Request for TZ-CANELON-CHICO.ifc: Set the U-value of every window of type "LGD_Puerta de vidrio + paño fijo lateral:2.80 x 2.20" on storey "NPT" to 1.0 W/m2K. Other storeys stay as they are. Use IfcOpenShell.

First a look at what the model holds.

```python
import ifcopenshell
import ifcopenshell.util.element

model = ifcopenshell.open("TZ-CANELON-CHICO.ifc")
print(model.schema)
storey = next(s for s in model.by_type("IfcBuildingStorey") if s.Name == "NPT")
windows = [e for e in ifcopenshell.util.element.get_decomposition(storey) if e.is_a("IfcWindow")]
seen = {}
for e in windows:
    element_type = ifcopenshell.util.element.get_type(e)
    key = (element_type.Name if element_type != e and element_type else None, ifcopenshell.util.element.get_pset(e, "Pset_WindowCommon", "ThermalTransmittance"))
    seen[key] = seen.get(key, 0) + 1
for (name, value), count in sorted(seen.items(), key=str):
    print(count, "x", name, "|", value)
```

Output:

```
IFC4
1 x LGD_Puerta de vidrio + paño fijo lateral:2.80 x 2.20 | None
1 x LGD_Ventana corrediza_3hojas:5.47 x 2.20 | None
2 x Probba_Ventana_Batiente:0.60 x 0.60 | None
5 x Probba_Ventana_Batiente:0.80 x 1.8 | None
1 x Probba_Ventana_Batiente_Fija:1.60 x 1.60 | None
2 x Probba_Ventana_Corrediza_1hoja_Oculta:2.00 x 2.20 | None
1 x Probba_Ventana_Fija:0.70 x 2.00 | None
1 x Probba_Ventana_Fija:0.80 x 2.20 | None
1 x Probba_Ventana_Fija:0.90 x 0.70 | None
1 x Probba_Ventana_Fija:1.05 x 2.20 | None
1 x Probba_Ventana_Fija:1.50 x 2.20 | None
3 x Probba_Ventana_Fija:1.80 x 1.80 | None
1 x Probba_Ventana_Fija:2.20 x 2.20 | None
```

```python
import ifcopenshell
import ifcopenshell.api.pset
import ifcopenshell.util.element

model = ifcopenshell.open("TZ-CANELON-CHICO.ifc")

storey = next(s for s in model.by_type("IfcBuildingStorey") if s.Name == "NPT")
windows = [e for e in ifcopenshell.util.element.get_decomposition(storey) if e.is_a("IfcWindow")]

count = 0
for e in windows:
    element_type = ifcopenshell.util.element.get_type(e)
    if element_type in (None, e) or element_type.Name != "LGD_Puerta de vidrio + paño fijo lateral:2.80 x 2.20":
        continue
    # add_pset returns the element's existing set when there is one.
    pset = ifcopenshell.api.pset.add_pset(model, product=e, name="Pset_WindowCommon")
    ifcopenshell.api.pset.edit_pset(model, pset=pset, properties={"ThermalTransmittance": 1.0})
    count += 1

print(count, "windows updated")

model.write("TZ-CANELON-CHICO_updated.ifc")
```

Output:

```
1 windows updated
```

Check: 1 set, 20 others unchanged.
